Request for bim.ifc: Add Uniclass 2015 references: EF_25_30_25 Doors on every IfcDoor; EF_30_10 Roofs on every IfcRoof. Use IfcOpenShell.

First a look at what the model holds.

```python
import ifcopenshell

model = ifcopenshell.open("bim.ifc")
print(model.schema)
print("classifications:", [c.Name for c in model.by_type("IfcClassification")])
for ifc_class in ("IfcDoor", "IfcRoof", "IfcStair", "IfcWall", "IfcWindow"):
    print(ifc_class, len(model.by_type(ifc_class)))
```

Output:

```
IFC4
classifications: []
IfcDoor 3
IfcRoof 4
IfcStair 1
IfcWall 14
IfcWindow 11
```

```python
import ifcopenshell
import ifcopenshell.api.classification

model = ifcopenshell.open("bim.ifc")

system = ifcopenshell.api.classification.add_classification(model, classification="Uniclass 2015")

codes = {
    "IfcDoor": ("EF_25_30_25", "Doors"),
    "IfcRoof": ("EF_30_10", "Roofs"),
}
for ifc_class, (code, name) in codes.items():
    products = model.by_type(ifc_class)
    ifcopenshell.api.classification.add_reference(
        model, products=products, classification=system, identification=code, name=name
    )
    print(code, len(products))

model.write("bim_rev.ifc")
```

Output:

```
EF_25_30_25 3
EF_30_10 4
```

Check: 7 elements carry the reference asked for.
